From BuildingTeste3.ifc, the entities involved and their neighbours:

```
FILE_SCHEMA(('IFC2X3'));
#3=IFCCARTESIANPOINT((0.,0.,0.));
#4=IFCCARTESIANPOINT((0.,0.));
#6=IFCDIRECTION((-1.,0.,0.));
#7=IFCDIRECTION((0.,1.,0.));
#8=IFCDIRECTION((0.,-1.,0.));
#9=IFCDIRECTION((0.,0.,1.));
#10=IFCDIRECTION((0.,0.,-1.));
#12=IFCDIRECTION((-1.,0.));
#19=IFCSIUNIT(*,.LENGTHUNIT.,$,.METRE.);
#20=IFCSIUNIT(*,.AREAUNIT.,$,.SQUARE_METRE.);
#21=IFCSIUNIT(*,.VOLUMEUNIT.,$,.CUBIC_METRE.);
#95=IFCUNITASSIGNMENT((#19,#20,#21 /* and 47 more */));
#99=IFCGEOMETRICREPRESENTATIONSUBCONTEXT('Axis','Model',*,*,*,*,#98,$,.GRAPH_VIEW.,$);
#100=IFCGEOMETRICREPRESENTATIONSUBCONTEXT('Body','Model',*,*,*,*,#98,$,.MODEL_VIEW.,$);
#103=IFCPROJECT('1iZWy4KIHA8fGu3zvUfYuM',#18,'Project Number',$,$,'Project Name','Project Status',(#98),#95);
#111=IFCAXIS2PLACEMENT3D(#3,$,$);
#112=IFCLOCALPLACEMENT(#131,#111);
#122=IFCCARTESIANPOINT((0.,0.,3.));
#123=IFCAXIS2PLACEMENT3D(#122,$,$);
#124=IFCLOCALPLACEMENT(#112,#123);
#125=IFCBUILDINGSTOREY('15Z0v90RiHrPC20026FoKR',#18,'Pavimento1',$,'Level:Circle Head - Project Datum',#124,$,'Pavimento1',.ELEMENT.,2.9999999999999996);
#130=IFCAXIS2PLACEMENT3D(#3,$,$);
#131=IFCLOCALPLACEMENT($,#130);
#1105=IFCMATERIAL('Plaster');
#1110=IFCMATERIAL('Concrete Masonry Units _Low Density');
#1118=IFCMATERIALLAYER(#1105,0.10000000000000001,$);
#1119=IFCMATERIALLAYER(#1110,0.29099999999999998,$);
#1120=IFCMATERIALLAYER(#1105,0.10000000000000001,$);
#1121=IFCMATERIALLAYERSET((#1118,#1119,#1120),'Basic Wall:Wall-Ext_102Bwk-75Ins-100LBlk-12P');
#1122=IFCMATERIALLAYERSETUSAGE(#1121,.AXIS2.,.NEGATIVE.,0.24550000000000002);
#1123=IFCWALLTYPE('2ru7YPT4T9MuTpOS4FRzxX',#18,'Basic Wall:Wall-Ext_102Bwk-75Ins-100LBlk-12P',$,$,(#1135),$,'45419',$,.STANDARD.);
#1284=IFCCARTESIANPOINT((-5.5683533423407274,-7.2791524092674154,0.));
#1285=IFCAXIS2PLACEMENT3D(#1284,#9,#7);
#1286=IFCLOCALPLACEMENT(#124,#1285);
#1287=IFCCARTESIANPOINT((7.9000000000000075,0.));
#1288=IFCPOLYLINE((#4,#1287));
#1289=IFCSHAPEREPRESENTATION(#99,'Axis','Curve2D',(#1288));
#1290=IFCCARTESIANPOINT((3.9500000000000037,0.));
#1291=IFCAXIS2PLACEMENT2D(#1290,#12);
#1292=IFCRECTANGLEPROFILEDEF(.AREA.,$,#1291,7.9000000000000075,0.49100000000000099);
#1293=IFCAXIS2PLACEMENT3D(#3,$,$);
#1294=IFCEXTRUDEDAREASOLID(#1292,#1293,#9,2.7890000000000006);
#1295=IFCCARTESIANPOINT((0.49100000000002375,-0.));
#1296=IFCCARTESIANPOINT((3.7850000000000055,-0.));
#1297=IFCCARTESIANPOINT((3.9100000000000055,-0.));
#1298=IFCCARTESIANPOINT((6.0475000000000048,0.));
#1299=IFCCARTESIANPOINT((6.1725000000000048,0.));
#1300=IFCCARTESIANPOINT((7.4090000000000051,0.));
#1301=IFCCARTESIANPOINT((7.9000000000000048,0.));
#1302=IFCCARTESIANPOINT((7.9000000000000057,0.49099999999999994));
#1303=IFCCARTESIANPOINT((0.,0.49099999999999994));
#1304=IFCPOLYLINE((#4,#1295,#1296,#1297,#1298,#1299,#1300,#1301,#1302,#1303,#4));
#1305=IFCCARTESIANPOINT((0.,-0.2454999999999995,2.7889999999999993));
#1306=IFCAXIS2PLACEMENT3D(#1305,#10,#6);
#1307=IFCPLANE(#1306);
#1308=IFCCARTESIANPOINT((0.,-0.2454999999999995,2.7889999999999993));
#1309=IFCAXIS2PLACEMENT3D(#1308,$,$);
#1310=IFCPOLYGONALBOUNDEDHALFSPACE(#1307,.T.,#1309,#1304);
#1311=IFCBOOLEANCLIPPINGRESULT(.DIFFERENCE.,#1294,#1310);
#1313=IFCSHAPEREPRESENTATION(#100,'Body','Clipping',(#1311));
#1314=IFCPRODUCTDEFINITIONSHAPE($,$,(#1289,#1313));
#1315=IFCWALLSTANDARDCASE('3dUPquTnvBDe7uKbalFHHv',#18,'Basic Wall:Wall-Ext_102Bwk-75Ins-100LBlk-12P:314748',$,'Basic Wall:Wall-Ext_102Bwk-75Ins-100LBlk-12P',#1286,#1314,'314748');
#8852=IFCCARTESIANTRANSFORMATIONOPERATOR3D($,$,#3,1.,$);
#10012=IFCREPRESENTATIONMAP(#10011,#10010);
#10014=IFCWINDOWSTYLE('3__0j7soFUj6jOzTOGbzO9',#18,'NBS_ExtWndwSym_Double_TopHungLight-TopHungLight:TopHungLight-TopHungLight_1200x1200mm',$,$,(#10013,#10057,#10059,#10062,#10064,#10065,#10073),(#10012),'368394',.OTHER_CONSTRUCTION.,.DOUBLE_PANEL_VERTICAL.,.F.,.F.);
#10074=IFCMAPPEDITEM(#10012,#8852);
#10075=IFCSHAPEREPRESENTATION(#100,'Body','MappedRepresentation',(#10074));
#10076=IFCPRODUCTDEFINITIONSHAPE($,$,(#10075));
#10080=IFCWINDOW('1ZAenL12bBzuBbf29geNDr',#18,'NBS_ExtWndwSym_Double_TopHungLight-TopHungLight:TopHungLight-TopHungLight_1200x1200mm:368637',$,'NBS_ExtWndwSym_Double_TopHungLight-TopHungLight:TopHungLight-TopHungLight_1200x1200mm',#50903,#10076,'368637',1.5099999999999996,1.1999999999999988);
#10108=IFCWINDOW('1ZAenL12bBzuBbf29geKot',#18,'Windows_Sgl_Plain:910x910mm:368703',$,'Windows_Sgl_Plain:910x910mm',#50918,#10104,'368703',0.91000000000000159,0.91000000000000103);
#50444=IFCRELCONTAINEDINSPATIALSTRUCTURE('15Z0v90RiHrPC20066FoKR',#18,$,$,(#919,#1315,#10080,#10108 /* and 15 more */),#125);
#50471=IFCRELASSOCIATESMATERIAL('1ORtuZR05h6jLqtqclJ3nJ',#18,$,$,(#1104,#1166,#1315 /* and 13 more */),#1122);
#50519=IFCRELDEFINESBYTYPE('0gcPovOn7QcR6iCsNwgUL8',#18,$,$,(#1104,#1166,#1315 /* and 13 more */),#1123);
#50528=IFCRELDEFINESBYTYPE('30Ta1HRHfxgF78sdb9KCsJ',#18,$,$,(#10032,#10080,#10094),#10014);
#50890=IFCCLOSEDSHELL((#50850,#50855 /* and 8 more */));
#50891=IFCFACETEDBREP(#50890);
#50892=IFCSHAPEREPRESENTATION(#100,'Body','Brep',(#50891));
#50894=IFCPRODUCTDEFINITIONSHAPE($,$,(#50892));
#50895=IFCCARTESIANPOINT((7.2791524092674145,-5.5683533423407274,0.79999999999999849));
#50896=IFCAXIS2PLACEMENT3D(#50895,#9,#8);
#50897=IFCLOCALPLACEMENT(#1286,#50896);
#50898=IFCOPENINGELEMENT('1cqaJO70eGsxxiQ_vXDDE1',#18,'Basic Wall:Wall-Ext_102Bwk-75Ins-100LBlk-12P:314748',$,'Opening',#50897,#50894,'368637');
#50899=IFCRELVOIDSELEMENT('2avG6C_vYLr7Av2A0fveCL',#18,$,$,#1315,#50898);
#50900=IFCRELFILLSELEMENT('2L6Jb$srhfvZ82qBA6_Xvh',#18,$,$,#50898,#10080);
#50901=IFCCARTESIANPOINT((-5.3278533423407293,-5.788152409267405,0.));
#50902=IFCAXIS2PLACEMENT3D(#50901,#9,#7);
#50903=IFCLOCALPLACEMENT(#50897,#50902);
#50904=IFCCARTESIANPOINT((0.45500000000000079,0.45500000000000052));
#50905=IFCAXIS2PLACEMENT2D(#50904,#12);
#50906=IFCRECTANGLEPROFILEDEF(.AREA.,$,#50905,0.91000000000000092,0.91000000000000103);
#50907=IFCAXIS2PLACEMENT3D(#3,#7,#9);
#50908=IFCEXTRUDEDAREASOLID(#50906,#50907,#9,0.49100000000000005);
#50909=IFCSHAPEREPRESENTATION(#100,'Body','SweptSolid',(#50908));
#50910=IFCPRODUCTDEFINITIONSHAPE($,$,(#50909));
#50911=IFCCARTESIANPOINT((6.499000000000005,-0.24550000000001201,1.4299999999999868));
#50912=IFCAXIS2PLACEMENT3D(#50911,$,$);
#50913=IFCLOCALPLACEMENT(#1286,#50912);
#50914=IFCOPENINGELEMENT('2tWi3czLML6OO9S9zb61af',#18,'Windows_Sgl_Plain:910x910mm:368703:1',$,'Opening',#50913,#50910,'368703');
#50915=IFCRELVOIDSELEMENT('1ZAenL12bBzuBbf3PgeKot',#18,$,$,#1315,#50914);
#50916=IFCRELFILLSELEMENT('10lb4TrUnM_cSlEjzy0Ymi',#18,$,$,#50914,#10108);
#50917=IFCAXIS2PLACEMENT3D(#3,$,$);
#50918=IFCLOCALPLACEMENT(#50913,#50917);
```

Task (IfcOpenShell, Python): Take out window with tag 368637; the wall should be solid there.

```python
import ifcopenshell
import ifcopenshell.api.feature
import ifcopenshell.api.root
import ifcopenshell.geom
import ifcopenshell.util.shape

model = ifcopenshell.open("BuildingTeste3.ifc")
settings = ifcopenshell.geom.settings()


def volume(element):
    """Net volume in cubic metres, openings subtracted."""
    shape = ifcopenshell.geom.create_shape(settings, element)
    return ifcopenshell.util.shape.get_volume(shape.geometry)


window = model.by_guid("1ZAenL12bBzuBbf29geNDr")
opening = window.FillsVoids[0].RelatingOpeningElement
wall = opening.VoidsElements[0].RelatingBuildingElement
before = volume(wall)

ifcopenshell.api.root.remove_product(model, product=window)
ifcopenshell.api.feature.remove_feature(model, feature=opening)

after = volume(wall)

print(f"wall volume {before:.3f} -> {after:.3f} m3")

model.write("BuildingTeste3_updated.ifc")
```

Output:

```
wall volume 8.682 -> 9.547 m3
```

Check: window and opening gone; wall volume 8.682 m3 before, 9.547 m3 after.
